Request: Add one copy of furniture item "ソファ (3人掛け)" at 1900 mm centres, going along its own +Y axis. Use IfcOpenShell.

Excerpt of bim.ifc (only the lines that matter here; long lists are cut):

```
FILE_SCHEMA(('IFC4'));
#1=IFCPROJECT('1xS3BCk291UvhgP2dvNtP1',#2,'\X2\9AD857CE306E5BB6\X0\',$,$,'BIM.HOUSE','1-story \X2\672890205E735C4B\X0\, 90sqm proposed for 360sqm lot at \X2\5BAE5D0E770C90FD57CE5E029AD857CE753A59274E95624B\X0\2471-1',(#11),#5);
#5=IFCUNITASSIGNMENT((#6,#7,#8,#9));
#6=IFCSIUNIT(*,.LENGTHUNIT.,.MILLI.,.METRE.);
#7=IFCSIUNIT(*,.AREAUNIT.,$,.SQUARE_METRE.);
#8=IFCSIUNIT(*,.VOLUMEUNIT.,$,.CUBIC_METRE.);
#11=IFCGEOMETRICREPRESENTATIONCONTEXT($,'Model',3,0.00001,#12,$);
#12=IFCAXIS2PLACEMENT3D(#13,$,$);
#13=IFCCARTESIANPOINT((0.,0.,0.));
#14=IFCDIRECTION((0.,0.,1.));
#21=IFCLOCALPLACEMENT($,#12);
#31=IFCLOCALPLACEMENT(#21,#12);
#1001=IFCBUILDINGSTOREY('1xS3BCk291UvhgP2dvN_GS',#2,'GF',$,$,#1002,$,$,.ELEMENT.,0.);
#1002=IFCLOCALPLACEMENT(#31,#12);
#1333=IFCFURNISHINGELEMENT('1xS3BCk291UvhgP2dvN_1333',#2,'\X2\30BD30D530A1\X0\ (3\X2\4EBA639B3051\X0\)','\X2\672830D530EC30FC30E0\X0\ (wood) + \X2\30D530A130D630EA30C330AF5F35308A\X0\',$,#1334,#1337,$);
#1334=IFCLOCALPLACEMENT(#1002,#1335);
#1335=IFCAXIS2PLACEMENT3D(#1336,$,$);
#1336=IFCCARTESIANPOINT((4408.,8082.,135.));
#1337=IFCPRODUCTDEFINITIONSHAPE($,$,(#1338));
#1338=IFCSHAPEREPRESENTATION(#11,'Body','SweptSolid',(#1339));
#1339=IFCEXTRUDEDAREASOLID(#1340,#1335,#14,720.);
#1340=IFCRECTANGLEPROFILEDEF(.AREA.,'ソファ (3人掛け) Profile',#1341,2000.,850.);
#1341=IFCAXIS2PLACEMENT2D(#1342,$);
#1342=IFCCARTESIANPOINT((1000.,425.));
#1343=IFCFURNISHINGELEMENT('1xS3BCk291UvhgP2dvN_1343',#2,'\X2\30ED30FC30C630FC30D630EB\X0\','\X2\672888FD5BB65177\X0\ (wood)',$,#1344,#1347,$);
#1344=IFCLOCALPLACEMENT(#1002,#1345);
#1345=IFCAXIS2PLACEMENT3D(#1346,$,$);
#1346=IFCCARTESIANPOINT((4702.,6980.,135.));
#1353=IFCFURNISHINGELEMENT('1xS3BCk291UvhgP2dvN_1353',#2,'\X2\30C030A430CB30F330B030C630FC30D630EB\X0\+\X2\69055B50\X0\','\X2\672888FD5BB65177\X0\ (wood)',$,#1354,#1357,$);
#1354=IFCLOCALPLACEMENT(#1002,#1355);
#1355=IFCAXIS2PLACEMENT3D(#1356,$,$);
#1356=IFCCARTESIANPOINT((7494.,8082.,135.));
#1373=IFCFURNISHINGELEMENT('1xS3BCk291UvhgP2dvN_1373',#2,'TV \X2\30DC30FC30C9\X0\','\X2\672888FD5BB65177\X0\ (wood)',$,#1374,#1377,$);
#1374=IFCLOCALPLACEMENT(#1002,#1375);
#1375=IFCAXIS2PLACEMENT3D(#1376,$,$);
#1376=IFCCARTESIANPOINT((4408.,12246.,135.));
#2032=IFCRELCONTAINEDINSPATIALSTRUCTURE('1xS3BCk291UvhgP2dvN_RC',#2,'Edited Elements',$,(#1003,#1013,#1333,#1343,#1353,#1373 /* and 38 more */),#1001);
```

```python
import ifcopenshell
import ifcopenshell.api.geometry
import ifcopenshell.api.root
import ifcopenshell.util.element
import ifcopenshell.util.placement
import ifcopenshell.util.unit

model = ifcopenshell.open("bim.ifc")
unit_scale = ifcopenshell.util.unit.calculate_unit_scale(model)


def reuse_history(source, copy):
    """copy_class also copies each property set's owner history, people and application; keep the originals."""
    for rel in copy.IsDefinedBy:
        if rel.is_a("IfcRelDefinesByProperties") and (history := rel.RelatingPropertyDefinition.OwnerHistory):
            rel.RelatingPropertyDefinition.OwnerHistory = source.OwnerHistory
            ifcopenshell.util.element.remove_deep2(model, history)


source = model.by_guid("1xS3BCk291UvhgP2dvN_1333")
base = ifcopenshell.util.placement.get_local_placement(source.ObjectPlacement)
step = base[:3, 1] * 1.9 / unit_scale

for i in range(1, 2):
    copy = ifcopenshell.api.root.copy_class(model, product=source)
    copy.Representation = ifcopenshell.util.element.copy_deep(
        model, source.Representation, exclude=["IfcGeometricRepresentationContext", "IfcRepresentationMap"]
    )
    reuse_history(source, copy)
    matrix = base.copy()
    matrix[:3, 3] += i * step
    print("added at", matrix[:3, 3].round(3) + 0.0)
    ifcopenshell.api.geometry.edit_object_placement(model, product=copy, matrix=matrix, is_si=False)

model.write("bim_edited.ifc")
```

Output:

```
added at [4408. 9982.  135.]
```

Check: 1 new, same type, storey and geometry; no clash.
